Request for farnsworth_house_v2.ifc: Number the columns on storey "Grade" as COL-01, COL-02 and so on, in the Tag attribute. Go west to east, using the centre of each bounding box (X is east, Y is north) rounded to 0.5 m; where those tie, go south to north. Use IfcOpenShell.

First a look at what the model holds.

```python
import ifcopenshell
import ifcopenshell.util.element
import ifcopenshell.util.placement

model = ifcopenshell.open("farnsworth_house_v2.ifc")
print(model.schema)
storey = next(s for s in model.by_type("IfcBuildingStorey") if s.Name == "Grade")
columns = [e for e in ifcopenshell.util.element.get_decomposition(storey) if e.is_a("IfcColumn")]
for e in sorted(columns, key=lambda e: e.id()):
    origin = ifcopenshell.util.placement.get_local_placement(e.ObjectPlacement)[:3, 3]
    print(e.id(), e.Tag, e.Name, origin.round(2) + 0.0, sep=" | ")
```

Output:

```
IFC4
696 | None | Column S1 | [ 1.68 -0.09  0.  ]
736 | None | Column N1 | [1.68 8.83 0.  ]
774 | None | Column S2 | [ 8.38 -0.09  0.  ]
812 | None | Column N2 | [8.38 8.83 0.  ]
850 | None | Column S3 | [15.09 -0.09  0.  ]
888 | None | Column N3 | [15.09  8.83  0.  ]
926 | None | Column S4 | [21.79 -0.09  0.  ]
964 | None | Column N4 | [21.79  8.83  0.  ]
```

```python
import ifcopenshell
import ifcopenshell.geom
import ifcopenshell.util.element
import ifcopenshell.util.shape

model = ifcopenshell.open("farnsworth_house_v2.ifc")
settings = ifcopenshell.geom.settings()
settings.set("use-world-coords", True)


def centre(element):
    shape = ifcopenshell.geom.create_shape(settings, element)
    return ifcopenshell.util.shape.get_bbox_centroid(shape.geometry)


storey = next(s for s in model.by_type("IfcBuildingStorey") if s.Name == "Grade")
columns = [e for e in ifcopenshell.util.element.get_decomposition(storey) if e.is_a("IfcColumn")]

# Insertion points can sit at a corner or the storey origin, so sort by the geometry (in metres).
centres = {e: centre(e) for e in columns}
columns.sort(key=lambda e: (round(centres[e][0] / 0.5), centres[e][1]))

for i, e in enumerate(columns, start=1):
    number = f"COL-{i:02d}"
    e.Tag = number
    print(e.id(), number)

model.write("farnsworth_house_v2_edited.ifc")
```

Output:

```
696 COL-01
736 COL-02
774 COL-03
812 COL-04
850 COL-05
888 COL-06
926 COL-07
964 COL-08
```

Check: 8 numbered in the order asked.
